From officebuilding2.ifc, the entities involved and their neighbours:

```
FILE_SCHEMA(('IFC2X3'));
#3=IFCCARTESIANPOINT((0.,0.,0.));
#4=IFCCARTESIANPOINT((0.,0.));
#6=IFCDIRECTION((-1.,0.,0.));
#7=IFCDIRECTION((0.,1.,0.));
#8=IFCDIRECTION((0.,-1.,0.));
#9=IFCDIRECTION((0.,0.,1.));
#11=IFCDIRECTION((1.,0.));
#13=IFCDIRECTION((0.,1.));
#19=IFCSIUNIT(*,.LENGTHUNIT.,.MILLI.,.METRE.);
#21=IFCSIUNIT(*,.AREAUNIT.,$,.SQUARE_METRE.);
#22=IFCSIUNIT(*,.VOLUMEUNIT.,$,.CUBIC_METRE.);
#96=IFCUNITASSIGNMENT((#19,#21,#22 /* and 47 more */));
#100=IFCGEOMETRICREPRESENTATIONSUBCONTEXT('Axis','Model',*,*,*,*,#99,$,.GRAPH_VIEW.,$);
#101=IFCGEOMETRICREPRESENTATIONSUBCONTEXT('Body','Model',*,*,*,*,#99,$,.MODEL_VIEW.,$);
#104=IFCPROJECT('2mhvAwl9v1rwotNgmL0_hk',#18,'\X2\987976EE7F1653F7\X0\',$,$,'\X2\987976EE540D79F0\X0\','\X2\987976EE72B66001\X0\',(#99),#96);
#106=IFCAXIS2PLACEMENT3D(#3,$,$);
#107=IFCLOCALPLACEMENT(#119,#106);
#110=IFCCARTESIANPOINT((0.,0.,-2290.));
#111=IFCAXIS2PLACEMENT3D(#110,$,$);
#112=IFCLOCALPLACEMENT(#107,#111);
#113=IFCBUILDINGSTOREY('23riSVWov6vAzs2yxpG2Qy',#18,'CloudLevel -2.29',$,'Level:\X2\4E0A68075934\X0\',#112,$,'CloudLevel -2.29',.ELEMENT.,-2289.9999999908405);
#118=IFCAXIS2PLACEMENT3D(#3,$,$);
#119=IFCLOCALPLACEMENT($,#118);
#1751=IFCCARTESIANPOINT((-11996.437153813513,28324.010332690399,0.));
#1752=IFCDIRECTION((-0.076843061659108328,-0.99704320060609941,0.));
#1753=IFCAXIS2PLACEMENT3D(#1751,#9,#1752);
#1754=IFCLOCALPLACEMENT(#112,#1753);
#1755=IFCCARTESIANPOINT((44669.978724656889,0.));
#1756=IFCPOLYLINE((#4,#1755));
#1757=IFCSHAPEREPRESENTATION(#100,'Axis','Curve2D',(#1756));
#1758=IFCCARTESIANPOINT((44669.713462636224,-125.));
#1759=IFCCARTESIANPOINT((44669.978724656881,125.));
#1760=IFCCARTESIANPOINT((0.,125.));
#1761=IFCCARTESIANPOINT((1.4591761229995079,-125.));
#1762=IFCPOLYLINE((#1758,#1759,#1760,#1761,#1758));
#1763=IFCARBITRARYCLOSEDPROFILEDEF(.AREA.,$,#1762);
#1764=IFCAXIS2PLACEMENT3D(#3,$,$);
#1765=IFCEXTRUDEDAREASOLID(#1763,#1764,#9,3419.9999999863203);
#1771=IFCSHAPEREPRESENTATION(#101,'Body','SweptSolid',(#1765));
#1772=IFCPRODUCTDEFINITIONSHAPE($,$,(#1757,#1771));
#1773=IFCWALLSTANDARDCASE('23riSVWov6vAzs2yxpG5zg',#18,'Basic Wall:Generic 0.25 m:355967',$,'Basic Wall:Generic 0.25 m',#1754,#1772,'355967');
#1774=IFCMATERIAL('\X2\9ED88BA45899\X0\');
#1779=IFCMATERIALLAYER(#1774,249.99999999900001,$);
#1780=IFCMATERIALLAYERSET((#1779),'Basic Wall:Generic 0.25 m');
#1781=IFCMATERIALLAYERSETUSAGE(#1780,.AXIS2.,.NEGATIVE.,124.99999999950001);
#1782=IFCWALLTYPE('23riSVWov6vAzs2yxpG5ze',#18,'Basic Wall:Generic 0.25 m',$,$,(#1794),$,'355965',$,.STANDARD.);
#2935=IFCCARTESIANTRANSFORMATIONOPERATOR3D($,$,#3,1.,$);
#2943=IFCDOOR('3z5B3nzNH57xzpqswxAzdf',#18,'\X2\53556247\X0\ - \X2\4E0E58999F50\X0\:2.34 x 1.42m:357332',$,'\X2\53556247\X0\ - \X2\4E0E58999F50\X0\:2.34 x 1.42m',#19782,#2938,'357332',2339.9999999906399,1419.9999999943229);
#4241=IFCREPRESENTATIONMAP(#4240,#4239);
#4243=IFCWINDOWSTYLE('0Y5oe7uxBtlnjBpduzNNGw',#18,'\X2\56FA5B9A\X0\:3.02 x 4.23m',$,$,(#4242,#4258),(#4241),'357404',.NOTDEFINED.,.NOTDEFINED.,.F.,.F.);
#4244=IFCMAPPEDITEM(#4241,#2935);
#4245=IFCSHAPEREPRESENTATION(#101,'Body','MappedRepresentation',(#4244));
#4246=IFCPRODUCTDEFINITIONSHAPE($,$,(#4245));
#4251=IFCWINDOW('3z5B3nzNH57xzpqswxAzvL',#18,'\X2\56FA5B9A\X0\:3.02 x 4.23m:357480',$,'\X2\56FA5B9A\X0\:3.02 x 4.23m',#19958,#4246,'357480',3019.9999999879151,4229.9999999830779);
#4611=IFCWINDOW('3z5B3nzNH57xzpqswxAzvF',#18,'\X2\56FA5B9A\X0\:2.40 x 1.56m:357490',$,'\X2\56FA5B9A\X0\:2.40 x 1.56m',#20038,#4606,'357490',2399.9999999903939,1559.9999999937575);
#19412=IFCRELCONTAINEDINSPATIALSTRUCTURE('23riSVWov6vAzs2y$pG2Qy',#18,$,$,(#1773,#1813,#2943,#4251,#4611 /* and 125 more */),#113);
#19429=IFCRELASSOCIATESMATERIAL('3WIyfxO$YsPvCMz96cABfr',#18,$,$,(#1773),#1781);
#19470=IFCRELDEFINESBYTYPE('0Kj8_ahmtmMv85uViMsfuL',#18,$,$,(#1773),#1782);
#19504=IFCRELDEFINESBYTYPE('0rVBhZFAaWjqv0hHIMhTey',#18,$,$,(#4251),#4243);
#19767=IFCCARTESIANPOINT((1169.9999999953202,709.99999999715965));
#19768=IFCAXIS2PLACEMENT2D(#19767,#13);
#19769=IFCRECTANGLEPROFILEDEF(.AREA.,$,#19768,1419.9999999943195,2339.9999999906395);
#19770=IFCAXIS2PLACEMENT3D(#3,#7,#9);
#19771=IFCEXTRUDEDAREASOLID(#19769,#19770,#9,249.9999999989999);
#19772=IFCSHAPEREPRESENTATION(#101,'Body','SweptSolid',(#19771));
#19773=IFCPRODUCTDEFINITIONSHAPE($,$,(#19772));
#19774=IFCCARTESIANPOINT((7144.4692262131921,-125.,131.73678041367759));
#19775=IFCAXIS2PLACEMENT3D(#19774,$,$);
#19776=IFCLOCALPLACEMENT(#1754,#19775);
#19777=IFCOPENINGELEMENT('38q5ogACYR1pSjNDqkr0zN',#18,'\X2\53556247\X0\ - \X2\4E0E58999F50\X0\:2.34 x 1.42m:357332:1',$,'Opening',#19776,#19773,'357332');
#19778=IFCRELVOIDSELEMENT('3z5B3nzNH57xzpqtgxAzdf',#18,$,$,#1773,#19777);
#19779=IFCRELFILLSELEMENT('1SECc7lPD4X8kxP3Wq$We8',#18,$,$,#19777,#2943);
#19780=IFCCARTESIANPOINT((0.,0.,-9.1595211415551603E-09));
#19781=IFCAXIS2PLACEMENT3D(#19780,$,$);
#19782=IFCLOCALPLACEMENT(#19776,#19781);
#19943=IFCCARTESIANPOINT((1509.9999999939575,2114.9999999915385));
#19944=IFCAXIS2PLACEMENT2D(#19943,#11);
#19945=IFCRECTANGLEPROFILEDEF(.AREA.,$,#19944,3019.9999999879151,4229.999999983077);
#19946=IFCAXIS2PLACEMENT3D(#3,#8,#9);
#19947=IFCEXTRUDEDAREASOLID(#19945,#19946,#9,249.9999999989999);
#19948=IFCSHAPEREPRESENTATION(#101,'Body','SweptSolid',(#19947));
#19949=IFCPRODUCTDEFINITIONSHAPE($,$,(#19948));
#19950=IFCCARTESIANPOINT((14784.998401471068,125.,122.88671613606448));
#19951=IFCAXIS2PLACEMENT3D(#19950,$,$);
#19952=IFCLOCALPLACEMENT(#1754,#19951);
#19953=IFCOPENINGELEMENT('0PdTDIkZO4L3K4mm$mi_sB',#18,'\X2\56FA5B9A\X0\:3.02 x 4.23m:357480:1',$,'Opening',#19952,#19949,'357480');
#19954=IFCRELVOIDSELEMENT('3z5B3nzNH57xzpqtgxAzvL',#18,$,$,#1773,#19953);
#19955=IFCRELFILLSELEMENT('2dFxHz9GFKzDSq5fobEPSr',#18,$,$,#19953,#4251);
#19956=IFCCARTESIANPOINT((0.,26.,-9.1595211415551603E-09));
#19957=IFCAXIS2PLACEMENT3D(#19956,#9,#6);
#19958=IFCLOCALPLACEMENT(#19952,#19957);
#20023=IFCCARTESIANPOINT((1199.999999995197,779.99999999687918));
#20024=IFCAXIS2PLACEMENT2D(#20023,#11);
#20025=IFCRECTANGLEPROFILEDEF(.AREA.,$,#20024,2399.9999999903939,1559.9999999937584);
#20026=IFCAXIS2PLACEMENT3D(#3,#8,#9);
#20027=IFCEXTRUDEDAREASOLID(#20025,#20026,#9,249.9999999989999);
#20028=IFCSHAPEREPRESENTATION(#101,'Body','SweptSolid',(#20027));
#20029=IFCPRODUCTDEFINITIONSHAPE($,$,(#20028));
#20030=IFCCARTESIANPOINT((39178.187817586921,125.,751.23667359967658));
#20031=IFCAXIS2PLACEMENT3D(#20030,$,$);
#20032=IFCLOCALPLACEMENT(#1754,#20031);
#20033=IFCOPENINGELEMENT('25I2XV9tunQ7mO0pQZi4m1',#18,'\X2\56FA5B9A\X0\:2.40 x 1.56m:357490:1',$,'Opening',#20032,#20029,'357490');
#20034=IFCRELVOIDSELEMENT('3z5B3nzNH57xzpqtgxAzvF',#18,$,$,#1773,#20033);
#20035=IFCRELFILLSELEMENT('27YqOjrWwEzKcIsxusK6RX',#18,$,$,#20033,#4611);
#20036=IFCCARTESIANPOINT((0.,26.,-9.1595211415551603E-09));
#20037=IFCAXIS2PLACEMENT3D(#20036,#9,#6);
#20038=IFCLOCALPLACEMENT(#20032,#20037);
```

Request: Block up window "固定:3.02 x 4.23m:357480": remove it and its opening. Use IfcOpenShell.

```python
import ifcopenshell
import ifcopenshell.api.feature
import ifcopenshell.api.root
import ifcopenshell.geom
import ifcopenshell.util.shape

model = ifcopenshell.open("officebuilding2.ifc")
settings = ifcopenshell.geom.settings()


def volume(element):
    """Net volume in cubic metres, openings subtracted."""
    shape = ifcopenshell.geom.create_shape(settings, element)
    return ifcopenshell.util.shape.get_volume(shape.geometry)


window = model.by_guid("3z5B3nzNH57xzpqswxAzvL")
opening = window.FillsVoids[0].RelatingOpeningElement
wall = opening.VoidsElements[0].RelatingBuildingElement
before = volume(wall)

ifcopenshell.api.root.remove_product(model, product=window)
ifcopenshell.api.feature.remove_feature(model, feature=opening)

after = volume(wall)

print(f"wall volume {before:.3f} -> {after:.3f} m3")

model.write("officebuilding2-out.ifc")
```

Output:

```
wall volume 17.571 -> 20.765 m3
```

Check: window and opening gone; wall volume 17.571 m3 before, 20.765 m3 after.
